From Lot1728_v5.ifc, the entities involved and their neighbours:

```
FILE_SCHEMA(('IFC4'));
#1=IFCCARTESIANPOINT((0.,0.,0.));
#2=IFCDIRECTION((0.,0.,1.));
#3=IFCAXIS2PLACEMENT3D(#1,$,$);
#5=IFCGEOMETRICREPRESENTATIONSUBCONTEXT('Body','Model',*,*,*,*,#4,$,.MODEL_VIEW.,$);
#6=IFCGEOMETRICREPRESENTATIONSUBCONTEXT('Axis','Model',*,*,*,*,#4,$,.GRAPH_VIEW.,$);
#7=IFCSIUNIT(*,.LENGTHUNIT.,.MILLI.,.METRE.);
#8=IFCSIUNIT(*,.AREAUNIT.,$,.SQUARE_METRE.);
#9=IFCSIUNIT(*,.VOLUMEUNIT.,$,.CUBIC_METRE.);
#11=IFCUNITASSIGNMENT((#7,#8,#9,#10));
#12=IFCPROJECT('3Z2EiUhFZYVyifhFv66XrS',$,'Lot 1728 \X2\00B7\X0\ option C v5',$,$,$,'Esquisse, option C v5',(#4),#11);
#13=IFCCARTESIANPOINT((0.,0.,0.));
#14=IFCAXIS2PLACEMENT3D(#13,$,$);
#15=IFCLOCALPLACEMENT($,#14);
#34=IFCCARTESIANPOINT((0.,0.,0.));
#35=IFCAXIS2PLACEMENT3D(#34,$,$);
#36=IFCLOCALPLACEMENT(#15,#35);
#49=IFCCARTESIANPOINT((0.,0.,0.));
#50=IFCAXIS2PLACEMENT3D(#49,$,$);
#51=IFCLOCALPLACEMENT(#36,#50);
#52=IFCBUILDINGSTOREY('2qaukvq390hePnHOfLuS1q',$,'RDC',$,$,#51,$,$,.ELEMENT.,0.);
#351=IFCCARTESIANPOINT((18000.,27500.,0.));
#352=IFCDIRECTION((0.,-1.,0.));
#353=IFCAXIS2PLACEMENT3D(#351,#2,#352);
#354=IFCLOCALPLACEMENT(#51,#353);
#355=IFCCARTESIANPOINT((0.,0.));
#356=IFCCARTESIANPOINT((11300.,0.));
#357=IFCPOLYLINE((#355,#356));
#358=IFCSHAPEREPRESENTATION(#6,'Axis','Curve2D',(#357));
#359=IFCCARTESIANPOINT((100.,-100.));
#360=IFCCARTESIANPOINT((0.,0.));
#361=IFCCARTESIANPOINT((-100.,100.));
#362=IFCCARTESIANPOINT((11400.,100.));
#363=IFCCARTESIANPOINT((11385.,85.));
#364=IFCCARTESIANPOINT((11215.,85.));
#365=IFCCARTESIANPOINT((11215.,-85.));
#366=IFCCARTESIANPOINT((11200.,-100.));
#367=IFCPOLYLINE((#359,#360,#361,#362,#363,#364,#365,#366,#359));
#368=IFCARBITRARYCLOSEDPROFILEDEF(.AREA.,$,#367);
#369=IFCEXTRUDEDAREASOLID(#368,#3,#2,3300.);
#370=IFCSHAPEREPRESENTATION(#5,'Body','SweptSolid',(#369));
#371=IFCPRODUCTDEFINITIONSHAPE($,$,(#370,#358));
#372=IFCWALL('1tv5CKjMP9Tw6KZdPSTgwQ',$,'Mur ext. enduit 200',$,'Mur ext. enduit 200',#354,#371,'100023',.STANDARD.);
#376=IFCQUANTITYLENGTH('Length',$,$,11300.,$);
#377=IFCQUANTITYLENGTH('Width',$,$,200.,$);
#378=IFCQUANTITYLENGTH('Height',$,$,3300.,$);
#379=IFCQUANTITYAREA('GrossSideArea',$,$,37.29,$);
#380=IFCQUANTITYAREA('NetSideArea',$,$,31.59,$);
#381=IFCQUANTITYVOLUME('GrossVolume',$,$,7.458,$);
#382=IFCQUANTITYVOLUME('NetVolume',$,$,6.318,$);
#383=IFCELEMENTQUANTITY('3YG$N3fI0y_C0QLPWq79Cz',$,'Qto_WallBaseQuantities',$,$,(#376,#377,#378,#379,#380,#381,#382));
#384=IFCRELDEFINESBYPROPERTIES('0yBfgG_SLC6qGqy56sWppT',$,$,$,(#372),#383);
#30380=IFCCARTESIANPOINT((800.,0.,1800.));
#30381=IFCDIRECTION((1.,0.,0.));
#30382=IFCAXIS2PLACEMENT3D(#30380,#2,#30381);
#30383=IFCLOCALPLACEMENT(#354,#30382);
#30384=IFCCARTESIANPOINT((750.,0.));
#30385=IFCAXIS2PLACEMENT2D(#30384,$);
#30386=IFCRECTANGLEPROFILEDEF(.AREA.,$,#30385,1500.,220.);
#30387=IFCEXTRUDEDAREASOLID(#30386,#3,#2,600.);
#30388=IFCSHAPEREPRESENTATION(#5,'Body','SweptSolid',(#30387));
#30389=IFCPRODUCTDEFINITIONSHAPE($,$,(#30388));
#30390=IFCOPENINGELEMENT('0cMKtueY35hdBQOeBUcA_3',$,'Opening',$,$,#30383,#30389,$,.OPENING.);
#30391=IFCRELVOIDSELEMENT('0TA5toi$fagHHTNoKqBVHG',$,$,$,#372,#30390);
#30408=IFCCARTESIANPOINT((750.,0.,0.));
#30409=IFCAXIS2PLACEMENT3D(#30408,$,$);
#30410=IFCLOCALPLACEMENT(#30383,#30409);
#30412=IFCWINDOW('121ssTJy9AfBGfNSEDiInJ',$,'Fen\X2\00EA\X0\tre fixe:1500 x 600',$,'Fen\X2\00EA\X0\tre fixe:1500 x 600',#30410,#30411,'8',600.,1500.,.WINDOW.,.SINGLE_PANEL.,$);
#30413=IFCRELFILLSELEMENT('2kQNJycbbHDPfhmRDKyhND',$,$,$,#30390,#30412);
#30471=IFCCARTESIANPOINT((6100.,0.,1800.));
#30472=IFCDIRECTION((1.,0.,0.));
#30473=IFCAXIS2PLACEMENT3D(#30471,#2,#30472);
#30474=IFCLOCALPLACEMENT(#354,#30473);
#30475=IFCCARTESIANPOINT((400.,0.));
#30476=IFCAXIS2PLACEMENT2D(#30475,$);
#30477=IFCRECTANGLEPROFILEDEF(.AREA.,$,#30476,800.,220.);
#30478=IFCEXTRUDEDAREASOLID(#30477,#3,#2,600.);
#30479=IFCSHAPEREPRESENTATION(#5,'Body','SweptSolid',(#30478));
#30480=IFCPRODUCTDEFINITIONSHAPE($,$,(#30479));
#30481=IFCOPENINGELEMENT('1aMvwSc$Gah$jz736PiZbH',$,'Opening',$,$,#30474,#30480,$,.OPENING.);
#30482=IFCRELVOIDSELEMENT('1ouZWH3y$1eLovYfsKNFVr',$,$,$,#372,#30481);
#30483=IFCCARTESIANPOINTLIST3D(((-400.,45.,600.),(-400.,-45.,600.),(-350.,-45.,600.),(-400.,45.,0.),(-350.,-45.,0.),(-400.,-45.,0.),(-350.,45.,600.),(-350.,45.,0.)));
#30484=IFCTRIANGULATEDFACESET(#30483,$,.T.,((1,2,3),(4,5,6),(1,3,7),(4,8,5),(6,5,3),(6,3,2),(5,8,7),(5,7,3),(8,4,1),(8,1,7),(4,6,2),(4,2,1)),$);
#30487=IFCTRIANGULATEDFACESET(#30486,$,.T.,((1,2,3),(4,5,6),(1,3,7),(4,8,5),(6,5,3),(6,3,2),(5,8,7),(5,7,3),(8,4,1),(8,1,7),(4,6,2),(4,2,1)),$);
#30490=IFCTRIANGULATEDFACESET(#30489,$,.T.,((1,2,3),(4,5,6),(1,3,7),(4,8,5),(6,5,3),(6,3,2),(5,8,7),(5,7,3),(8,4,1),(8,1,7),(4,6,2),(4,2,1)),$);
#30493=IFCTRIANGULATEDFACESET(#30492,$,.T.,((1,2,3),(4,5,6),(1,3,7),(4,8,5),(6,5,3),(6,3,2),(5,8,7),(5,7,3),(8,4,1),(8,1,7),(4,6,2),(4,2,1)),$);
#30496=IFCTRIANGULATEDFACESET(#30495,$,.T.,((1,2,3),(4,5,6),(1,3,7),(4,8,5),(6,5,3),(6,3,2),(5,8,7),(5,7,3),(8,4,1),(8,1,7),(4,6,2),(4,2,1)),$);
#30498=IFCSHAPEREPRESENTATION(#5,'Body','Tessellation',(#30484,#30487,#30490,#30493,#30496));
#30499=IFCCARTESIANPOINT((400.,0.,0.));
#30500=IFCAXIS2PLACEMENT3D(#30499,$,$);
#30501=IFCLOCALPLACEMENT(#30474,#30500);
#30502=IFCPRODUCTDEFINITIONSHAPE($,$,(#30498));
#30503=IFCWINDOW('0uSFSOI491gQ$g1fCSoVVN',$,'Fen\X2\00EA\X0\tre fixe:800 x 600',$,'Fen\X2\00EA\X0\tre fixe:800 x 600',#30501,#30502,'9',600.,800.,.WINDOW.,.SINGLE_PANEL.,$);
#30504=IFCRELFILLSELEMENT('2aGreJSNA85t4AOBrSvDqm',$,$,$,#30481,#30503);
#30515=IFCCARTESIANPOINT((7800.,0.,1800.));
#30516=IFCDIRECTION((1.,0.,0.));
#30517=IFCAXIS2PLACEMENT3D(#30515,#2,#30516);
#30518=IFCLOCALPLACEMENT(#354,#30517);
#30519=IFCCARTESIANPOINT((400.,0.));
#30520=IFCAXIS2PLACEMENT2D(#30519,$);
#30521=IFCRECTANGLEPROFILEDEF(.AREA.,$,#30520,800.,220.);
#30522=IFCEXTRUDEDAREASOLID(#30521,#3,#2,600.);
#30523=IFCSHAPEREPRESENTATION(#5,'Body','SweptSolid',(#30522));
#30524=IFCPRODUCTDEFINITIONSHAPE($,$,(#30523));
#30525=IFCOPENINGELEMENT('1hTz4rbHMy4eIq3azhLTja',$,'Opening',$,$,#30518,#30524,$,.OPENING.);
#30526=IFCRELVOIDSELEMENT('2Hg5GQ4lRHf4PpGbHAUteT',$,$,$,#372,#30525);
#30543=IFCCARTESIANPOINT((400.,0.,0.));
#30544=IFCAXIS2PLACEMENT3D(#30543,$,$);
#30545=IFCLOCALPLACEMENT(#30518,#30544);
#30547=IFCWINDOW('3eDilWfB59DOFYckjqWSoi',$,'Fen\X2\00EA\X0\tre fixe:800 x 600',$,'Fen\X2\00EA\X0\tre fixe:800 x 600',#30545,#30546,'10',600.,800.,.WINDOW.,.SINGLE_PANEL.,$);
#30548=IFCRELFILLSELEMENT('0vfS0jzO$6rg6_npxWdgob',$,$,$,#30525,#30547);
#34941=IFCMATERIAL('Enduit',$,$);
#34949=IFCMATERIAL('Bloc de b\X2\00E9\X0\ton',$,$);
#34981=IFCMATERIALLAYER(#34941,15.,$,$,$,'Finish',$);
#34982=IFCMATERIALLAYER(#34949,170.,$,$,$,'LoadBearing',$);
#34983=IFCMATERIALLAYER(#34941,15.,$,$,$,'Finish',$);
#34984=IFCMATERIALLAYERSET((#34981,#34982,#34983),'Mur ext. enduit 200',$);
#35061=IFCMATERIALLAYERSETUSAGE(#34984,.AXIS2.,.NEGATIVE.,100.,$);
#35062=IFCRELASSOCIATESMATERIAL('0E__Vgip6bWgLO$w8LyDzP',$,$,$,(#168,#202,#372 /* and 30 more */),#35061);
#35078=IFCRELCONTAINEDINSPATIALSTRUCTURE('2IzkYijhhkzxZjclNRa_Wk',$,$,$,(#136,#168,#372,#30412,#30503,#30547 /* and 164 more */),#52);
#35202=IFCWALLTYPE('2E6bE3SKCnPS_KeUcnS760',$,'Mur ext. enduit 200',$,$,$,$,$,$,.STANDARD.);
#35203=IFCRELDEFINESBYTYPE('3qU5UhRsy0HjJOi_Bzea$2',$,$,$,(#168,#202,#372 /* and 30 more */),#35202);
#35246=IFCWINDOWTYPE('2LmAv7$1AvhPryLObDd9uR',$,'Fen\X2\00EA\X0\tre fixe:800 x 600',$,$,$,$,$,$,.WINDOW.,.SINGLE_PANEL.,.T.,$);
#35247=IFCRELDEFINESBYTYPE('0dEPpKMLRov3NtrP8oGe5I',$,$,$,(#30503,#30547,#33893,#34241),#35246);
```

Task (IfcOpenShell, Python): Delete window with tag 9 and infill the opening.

```python
import ifcopenshell
import ifcopenshell.api.feature
import ifcopenshell.api.pset
import ifcopenshell.api.root
import ifcopenshell.geom
import ifcopenshell.util.element
import ifcopenshell.util.shape
import ifcopenshell.util.unit

model = ifcopenshell.open("Lot1728_v5.ifc")
area_scale = ifcopenshell.util.unit.calculate_unit_scale(model, "AREAUNIT")
volume_scale = ifcopenshell.util.unit.calculate_unit_scale(model, "VOLUMEUNIT")
settings = ifcopenshell.geom.settings()


def volume(element):
    """Net volume in cubic metres, openings subtracted."""
    shape = ifcopenshell.geom.create_shape(settings, element)
    return ifcopenshell.util.shape.get_volume(shape.geometry)


window = model.by_guid("0uSFSOI491gQ$g1fCSoVVN")
opening = window.FillsVoids[0].RelatingOpeningElement
wall = opening.VoidsElements[0].RelatingBuildingElement
before = volume(wall)

ifcopenshell.api.root.remove_product(model, product=window)
ifcopenshell.api.feature.remove_feature(model, feature=opening)

after = volume(wall)
thickness = 0.2  # wall thickness in metres

# Update the wall's stored quantities.
qto = model.by_id(ifcopenshell.util.element.get_pset(wall, "Qto_WallBaseQuantities", should_inherit=False)["id"])
ifcopenshell.api.pset.edit_qto(model, qto=qto, properties={
    "NetSideArea": after / thickness / area_scale,
    "NetVolume": after / volume_scale,
})

print(f"wall volume {before:.3f} -> {after:.3f} m3")

model.write("Lot1728_v5-out.ifc")
```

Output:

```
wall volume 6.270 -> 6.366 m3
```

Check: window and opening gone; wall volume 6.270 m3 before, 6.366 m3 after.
